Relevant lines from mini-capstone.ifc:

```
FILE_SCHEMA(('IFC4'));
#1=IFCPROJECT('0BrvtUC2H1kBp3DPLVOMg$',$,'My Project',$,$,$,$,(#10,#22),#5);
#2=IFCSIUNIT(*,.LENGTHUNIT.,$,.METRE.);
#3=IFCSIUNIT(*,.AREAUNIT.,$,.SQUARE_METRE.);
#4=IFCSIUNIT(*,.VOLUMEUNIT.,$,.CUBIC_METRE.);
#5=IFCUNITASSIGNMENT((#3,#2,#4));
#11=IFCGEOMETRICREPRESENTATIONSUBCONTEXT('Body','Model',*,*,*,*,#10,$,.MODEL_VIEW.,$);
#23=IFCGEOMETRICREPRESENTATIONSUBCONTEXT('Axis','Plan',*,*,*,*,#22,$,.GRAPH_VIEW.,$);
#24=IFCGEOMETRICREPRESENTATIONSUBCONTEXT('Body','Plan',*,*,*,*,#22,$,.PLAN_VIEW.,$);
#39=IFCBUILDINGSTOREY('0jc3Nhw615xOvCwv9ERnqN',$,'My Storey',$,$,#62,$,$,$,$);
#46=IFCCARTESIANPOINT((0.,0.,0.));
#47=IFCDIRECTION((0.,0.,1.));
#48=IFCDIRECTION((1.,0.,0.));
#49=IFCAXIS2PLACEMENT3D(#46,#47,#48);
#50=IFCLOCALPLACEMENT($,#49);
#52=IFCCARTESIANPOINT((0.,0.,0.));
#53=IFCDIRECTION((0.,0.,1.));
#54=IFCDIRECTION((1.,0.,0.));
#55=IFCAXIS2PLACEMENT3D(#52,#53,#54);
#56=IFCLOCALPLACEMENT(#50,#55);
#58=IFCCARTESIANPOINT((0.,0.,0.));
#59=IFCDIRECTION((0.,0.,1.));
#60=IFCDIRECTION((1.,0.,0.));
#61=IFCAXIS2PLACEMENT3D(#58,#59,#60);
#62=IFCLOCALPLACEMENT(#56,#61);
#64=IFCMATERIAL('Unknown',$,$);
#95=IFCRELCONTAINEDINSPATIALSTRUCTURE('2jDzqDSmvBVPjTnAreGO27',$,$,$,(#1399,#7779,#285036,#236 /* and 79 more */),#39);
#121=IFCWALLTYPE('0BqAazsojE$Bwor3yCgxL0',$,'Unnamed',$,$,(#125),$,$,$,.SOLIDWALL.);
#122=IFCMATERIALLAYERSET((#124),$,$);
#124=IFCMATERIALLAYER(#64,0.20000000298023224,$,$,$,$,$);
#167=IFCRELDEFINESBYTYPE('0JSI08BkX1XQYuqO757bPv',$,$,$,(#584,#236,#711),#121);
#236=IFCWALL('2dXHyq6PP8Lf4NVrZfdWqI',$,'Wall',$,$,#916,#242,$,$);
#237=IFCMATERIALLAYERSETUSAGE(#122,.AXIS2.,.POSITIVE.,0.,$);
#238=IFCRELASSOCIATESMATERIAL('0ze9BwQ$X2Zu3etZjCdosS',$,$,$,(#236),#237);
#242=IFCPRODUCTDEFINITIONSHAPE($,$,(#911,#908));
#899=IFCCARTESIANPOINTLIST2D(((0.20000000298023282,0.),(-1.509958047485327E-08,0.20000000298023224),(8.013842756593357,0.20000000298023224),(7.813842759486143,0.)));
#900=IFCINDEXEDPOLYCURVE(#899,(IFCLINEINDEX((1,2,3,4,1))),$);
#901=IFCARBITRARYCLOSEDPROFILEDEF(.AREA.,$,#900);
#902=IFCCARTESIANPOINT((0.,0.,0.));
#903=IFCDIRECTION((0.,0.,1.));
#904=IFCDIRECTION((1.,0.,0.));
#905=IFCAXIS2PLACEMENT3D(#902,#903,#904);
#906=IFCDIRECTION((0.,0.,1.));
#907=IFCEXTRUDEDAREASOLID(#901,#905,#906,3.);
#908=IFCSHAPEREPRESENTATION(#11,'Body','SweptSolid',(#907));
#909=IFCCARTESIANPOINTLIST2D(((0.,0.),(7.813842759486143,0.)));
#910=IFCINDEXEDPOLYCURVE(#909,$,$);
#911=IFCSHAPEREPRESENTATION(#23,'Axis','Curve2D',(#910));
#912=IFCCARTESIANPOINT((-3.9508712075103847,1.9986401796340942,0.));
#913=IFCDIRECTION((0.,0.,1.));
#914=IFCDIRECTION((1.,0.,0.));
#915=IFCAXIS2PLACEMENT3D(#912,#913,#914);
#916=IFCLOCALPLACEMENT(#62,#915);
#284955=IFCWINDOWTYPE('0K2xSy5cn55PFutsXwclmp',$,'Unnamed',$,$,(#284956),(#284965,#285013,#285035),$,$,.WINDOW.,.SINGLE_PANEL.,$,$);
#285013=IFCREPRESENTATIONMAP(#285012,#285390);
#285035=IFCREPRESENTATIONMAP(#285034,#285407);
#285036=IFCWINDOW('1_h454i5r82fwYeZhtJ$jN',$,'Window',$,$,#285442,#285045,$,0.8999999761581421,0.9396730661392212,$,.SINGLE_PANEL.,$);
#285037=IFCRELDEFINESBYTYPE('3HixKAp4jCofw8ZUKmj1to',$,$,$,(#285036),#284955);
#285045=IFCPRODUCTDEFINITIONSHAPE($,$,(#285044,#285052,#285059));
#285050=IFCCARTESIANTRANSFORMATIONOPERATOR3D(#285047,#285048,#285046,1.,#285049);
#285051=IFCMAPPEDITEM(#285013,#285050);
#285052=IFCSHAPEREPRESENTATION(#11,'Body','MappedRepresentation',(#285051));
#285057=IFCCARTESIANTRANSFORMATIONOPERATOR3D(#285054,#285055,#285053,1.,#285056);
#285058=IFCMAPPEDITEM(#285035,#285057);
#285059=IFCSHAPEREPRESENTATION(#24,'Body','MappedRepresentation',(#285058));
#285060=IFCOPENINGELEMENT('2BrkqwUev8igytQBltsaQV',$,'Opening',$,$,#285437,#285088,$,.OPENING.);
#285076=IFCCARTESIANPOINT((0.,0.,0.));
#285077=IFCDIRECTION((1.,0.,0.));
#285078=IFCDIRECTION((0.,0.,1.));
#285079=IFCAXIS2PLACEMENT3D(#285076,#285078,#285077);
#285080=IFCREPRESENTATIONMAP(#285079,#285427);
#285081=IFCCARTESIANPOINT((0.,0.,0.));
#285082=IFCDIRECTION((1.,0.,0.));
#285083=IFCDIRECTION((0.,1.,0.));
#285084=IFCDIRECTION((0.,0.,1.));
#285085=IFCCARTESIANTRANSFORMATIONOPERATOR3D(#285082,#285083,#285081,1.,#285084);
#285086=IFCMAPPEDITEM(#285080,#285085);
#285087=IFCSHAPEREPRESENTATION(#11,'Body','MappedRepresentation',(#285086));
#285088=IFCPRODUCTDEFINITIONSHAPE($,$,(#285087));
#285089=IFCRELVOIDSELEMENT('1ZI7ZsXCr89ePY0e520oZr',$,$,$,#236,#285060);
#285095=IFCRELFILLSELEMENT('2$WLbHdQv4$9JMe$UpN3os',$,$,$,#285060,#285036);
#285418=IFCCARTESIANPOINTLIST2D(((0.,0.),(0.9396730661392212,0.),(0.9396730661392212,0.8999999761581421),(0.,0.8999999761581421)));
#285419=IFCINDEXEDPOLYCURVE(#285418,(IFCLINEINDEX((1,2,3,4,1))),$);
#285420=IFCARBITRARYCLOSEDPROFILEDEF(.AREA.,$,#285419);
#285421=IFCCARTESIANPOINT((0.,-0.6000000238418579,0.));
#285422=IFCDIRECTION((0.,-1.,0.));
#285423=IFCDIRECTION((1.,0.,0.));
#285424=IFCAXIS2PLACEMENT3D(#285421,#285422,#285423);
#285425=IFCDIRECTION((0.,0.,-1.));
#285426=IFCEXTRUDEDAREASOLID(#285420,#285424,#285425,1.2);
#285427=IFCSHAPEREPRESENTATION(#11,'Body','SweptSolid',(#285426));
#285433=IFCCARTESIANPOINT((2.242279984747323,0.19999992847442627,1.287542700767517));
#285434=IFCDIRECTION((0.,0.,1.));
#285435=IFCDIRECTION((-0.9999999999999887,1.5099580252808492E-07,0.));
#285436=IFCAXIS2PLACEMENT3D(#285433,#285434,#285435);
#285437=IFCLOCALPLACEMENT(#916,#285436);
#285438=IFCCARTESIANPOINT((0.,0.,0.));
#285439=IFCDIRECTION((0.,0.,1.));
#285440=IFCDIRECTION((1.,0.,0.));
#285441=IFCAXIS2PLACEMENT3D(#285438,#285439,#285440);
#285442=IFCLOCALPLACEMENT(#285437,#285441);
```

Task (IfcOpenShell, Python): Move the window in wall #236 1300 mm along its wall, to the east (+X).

```python
import ifcopenshell
import ifcopenshell.api.geometry
import ifcopenshell.util.placement

model = ifcopenshell.open("mini-capstone.ifc")

window = model.by_guid("1_h454i5r82fwYeZhtJ$jN")
opening = window.FillsVoids[0].RelatingOpeningElement
wall = opening.VoidsElements[0].RelatingBuildingElement

wall_matrix = ifcopenshell.util.placement.get_local_placement(wall.ObjectPlacement)
shift = wall_matrix[:3, 0] * 1.3
before = ifcopenshell.util.placement.get_local_placement(window.ObjectPlacement)[:3, 3].copy()

# The window is placed relative to its opening, so it follows when the opening moves.
matrix = ifcopenshell.util.placement.get_local_placement(opening.ObjectPlacement)
matrix[:3, 3] += shift
ifcopenshell.api.geometry.edit_object_placement(
    model, product=opening, matrix=matrix, is_si=False, should_transform_children=True
)

after = ifcopenshell.util.placement.get_local_placement(window.ObjectPlacement)[:3, 3]
print("window moved by", (after - before).round(3) + 0.0)

model.write("mini-capstone_edited.ifc")
```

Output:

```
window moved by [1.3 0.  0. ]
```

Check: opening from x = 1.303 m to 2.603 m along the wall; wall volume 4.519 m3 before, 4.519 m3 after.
